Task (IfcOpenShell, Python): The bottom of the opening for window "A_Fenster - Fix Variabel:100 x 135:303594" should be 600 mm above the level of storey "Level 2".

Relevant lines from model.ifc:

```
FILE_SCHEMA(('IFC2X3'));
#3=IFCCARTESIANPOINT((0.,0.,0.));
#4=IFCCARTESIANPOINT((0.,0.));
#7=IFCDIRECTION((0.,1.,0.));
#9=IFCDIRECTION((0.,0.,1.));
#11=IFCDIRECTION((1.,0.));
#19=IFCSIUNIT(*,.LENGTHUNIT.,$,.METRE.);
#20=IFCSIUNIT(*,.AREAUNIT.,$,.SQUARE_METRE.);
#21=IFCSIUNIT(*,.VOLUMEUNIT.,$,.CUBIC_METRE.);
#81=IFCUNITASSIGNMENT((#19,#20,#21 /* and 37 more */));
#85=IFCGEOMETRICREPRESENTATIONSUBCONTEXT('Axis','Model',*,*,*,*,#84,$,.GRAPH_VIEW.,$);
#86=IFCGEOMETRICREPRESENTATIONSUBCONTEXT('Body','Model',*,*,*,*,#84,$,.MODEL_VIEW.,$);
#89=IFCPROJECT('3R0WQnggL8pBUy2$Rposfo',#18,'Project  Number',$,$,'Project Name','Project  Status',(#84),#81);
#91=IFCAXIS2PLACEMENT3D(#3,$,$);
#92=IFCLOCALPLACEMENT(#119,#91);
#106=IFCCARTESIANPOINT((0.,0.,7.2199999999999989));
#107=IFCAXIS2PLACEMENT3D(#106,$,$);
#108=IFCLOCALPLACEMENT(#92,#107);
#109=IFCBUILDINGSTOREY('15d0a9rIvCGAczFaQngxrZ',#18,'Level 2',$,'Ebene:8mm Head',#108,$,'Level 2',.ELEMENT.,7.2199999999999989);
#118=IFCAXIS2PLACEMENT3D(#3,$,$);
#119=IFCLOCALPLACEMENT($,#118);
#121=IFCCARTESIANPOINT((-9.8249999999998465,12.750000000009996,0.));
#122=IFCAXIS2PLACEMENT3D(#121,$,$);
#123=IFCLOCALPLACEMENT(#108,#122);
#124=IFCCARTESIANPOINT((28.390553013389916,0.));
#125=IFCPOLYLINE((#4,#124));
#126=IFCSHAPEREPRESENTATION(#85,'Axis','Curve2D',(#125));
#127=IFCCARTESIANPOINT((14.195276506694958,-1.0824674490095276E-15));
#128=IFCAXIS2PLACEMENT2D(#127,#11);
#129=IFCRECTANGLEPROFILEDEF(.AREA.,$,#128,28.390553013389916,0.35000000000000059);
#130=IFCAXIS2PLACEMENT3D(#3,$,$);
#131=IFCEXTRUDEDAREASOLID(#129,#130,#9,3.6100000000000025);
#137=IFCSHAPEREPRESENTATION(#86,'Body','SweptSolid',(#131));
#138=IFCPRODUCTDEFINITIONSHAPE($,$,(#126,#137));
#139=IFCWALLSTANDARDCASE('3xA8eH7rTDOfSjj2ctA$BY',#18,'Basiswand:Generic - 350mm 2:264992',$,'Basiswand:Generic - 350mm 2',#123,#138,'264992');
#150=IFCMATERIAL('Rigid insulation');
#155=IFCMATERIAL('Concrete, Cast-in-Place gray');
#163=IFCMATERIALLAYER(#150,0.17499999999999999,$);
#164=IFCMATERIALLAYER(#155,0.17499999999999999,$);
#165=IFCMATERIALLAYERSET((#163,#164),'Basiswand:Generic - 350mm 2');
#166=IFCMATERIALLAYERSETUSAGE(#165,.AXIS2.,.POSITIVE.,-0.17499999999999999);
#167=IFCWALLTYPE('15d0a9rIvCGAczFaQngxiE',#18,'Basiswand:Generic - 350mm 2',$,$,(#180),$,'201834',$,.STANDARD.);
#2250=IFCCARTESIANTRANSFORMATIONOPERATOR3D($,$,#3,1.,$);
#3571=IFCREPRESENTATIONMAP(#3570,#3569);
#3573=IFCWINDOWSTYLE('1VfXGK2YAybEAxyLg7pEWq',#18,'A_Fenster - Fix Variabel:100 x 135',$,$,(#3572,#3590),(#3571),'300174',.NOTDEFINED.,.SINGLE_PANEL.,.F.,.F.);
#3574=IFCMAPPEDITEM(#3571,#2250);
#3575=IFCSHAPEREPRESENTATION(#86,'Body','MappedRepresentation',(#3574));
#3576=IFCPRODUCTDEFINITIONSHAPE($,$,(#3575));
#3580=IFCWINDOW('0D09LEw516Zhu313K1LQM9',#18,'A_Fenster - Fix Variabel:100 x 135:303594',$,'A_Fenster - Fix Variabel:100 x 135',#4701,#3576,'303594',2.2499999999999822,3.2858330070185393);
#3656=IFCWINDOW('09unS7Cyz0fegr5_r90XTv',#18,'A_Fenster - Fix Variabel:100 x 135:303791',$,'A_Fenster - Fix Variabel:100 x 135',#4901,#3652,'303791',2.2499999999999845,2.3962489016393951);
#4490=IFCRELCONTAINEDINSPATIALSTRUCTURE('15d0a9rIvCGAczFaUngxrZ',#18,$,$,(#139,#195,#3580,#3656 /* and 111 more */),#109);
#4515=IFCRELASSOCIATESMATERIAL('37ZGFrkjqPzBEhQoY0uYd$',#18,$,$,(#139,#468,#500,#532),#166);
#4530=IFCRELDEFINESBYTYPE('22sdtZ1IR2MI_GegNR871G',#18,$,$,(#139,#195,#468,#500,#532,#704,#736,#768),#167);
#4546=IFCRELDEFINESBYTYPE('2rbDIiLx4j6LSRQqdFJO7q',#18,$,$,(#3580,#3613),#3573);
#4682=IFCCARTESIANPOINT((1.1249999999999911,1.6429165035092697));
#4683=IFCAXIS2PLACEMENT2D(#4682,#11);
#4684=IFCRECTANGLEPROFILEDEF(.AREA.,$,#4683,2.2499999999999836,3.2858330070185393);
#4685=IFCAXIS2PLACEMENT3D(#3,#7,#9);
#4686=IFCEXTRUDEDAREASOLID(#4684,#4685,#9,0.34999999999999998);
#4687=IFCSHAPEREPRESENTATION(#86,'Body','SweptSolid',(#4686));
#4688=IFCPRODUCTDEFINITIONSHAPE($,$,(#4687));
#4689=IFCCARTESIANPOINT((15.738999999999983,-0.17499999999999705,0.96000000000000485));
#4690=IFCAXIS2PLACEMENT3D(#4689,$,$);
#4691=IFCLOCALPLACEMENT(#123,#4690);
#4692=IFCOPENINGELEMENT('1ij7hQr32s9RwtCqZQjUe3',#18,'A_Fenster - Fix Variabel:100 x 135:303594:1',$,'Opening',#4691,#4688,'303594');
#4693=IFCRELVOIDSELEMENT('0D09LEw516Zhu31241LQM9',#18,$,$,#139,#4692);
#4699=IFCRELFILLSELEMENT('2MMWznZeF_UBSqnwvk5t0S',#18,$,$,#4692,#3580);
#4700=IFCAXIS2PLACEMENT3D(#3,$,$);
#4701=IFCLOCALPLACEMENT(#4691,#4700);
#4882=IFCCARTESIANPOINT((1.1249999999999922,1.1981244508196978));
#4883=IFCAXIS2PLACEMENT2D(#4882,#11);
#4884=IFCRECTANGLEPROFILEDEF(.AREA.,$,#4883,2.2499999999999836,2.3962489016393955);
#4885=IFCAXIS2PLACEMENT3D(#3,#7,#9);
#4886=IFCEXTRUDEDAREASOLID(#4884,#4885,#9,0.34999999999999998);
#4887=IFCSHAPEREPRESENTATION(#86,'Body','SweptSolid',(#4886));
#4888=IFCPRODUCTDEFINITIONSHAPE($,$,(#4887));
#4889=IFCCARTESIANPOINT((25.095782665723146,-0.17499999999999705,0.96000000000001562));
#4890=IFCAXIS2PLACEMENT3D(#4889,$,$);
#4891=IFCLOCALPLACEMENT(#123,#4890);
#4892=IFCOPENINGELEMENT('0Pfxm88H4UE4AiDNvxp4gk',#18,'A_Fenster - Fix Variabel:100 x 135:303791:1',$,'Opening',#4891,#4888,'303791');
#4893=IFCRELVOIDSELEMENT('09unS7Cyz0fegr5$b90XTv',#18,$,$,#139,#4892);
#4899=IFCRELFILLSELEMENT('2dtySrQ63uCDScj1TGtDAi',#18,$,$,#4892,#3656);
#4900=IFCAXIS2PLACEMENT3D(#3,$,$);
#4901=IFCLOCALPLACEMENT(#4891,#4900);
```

```python
import numpy as np
import ifcopenshell
import ifcopenshell.api.geometry
import ifcopenshell.geom
import ifcopenshell.util.element
import ifcopenshell.util.placement
import ifcopenshell.util.shape
import ifcopenshell.util.unit

model = ifcopenshell.open("model.ifc")
unit_scale = ifcopenshell.util.unit.calculate_unit_scale(model)

window = model.by_id(3580)
opening = window.FillsVoids[0].RelatingOpeningElement
storey = ifcopenshell.util.element.get_container(window, ifc_class="IfcBuildingStorey")
level = ifcopenshell.util.placement.get_local_placement(storey.ObjectPlacement)[2, 3]

# The opening's origin need not be at the sill, so measure its lowest point.
shape = ifcopenshell.geom.create_shape(ifcopenshell.geom.settings(), opening)
bottom = ifcopenshell.util.shape.get_shape_bottom_elevation(shape, shape.geometry) / unit_scale
dz = level + 0.6 - bottom

shift = np.array([0.0, 0.0, dz])
# The window is placed relative to its opening, so it follows when the opening moves.
matrix = ifcopenshell.util.placement.get_local_placement(opening.ObjectPlacement)
matrix[:3, 3] += shift
ifcopenshell.api.geometry.edit_object_placement(
    model, product=opening, matrix=matrix, is_si=False, should_transform_children=True
)

print(f"moved by {dz * unit_scale:+.3f} m")

model.write("model-out.ifc")
```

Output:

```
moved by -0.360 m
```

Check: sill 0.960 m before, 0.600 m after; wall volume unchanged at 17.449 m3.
